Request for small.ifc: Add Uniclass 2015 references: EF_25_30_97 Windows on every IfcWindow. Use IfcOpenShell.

First a look at what the model holds.

```python
import ifcopenshell

model = ifcopenshell.open("small.ifc")
print(model.schema)
print("classifications:", [c.Name for c in model.by_type("IfcClassification")])
for ifc_class in ("IfcDoor", "IfcRoof", "IfcStair", "IfcWall", "IfcWindow"):
    print(ifc_class, len(model.by_type(ifc_class)))
```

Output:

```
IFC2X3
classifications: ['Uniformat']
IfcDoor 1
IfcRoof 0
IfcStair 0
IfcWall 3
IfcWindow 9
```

```python
import ifcopenshell
import ifcopenshell.api.classification

model = ifcopenshell.open("small.ifc")

# IFC2X3 requires Source and Edition and has no link from the project to the system.
system = model.create_entity("IfcClassification", Source="NBS", Edition="2015", Name="Uniclass 2015")

codes = {
    "IfcWindow": ("EF_25_30_97", "Windows"),
}
for ifc_class, (code, name) in codes.items():
    products = model.by_type(ifc_class)
    ifcopenshell.api.classification.add_reference(
        model, products=products, classification=system, identification=code, name=name
    )
    print(code, len(products))

model.write("small_rev.ifc")
```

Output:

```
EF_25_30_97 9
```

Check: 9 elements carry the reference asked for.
